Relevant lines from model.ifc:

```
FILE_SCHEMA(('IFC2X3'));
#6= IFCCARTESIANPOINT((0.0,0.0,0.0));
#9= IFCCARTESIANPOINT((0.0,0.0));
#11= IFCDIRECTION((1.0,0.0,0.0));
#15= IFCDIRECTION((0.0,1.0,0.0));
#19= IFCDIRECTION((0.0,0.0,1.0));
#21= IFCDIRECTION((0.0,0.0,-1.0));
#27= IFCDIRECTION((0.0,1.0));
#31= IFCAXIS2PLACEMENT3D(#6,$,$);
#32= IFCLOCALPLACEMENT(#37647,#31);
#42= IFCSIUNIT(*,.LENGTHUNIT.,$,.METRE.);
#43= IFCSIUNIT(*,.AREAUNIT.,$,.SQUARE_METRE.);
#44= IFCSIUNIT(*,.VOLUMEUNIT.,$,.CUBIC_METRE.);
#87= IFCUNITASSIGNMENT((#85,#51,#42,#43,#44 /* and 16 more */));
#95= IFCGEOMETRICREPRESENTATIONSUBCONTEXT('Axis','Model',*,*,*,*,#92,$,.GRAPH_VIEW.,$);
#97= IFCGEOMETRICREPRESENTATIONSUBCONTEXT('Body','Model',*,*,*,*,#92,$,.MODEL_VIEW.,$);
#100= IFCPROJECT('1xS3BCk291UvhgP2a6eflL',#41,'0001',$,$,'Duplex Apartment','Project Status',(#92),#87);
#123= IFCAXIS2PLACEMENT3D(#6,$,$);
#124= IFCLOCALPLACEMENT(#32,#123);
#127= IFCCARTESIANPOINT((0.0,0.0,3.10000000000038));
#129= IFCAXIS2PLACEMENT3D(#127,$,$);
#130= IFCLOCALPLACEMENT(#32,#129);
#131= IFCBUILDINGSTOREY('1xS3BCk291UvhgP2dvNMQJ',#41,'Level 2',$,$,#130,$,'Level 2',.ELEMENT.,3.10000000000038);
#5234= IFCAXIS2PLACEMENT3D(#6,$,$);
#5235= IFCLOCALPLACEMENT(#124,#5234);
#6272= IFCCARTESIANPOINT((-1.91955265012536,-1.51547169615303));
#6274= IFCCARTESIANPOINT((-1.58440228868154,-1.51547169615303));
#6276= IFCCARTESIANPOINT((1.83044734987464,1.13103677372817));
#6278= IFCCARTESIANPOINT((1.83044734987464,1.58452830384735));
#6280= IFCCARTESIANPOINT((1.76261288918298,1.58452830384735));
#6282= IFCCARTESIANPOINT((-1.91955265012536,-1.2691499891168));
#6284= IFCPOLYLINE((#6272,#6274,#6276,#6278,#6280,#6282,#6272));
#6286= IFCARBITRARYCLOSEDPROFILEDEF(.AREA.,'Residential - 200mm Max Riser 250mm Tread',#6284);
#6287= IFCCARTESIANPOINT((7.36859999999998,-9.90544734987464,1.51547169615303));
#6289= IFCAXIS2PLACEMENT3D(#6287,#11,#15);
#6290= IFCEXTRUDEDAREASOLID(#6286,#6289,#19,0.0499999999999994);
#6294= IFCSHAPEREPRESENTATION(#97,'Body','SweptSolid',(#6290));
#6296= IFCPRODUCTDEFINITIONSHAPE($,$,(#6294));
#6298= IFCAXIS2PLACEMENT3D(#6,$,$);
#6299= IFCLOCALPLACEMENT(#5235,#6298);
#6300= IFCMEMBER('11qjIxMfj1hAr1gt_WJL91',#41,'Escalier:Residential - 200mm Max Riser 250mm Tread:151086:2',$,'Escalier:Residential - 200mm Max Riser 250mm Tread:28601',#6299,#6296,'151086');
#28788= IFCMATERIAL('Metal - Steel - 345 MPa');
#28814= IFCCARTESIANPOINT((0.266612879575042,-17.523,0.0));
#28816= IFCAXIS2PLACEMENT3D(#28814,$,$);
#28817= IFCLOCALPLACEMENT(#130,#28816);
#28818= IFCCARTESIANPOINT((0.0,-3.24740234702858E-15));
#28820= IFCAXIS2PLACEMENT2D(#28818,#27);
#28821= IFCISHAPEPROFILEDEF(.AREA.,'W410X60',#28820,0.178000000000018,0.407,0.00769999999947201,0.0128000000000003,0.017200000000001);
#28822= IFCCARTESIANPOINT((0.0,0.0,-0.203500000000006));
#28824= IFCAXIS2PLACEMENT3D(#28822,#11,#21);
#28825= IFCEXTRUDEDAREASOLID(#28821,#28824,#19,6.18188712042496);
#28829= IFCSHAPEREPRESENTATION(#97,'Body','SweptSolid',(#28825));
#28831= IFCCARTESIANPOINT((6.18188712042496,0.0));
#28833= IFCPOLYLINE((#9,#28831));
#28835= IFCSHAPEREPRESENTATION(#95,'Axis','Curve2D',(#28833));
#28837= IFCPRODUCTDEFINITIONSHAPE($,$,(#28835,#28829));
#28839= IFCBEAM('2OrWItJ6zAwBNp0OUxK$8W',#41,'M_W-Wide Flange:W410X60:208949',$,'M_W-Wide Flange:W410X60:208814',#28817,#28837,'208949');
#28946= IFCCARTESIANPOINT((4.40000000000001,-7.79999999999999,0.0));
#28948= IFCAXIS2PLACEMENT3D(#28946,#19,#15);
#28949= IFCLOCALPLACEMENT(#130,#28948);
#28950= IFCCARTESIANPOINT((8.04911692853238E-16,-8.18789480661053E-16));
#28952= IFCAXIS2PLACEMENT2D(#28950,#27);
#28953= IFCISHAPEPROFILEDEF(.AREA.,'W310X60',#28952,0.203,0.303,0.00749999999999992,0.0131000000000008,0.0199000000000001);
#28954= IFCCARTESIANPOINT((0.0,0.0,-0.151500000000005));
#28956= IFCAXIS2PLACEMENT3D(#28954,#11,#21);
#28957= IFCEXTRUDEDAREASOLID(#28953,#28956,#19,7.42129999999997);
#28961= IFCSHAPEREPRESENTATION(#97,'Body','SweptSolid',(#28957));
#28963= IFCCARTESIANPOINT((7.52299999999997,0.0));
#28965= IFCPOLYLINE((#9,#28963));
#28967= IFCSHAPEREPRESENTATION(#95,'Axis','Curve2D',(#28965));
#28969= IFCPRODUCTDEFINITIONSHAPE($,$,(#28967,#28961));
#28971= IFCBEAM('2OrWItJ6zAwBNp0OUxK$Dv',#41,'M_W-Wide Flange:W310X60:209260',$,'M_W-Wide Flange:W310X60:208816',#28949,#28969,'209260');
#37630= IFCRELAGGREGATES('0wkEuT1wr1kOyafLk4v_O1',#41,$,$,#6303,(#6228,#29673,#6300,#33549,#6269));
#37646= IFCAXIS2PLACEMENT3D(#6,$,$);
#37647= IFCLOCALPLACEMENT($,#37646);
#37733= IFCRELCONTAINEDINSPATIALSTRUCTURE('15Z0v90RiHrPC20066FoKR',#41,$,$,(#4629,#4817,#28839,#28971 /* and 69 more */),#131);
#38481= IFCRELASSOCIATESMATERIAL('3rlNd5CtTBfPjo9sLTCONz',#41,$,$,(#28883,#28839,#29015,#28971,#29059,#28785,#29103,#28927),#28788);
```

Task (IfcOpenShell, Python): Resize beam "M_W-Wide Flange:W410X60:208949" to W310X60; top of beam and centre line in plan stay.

```python
import ifcopenshell
import ifcopenshell.util.element
import ifcopenshell.util.representation

model = ifcopenshell.open("model.ifc")

member = model.by_id(28839)
source = next(p for p in model.by_type("IfcIShapeProfileDef") if p.ProfileName == "W310X60")

body = ifcopenshell.util.representation.get_representation(member, "Model", "Body")
solid = body.Items[0]
old_profile = solid.SweptArea

# Copy the section's sizes but keep this member's own profile position.
profile = ifcopenshell.util.element.copy(model, source)
# Profiles are centred, so shift by half the change in depth to hold the top.
shift = (old_profile.OverallDepth - profile.OverallDepth) / 2
x, y = old_profile.Position.Location.Coordinates
up = (-1.0, 0.0)  # upwards, in the solid's own plane
location = model.createIfcCartesianPoint((x + up[0] * shift, y + up[1] * shift))
profile.Position = model.createIfcAxis2Placement2D(location, old_profile.Position.RefDirection)
solid.SweptArea = profile
if not model.get_total_inverses(old_profile):
    ifcopenshell.util.element.remove_deep2(model, old_profile)
member.Name = member.Name.replace("W410X60", "W310X60")
member.ObjectType = member.ObjectType.replace("W410X60", "W310X60")

print(solid.SweptArea)

model.write("model_edited.ifc")
```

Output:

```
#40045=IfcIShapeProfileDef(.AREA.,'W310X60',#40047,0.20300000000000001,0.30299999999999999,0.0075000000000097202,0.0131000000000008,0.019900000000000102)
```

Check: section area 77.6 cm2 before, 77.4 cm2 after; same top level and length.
